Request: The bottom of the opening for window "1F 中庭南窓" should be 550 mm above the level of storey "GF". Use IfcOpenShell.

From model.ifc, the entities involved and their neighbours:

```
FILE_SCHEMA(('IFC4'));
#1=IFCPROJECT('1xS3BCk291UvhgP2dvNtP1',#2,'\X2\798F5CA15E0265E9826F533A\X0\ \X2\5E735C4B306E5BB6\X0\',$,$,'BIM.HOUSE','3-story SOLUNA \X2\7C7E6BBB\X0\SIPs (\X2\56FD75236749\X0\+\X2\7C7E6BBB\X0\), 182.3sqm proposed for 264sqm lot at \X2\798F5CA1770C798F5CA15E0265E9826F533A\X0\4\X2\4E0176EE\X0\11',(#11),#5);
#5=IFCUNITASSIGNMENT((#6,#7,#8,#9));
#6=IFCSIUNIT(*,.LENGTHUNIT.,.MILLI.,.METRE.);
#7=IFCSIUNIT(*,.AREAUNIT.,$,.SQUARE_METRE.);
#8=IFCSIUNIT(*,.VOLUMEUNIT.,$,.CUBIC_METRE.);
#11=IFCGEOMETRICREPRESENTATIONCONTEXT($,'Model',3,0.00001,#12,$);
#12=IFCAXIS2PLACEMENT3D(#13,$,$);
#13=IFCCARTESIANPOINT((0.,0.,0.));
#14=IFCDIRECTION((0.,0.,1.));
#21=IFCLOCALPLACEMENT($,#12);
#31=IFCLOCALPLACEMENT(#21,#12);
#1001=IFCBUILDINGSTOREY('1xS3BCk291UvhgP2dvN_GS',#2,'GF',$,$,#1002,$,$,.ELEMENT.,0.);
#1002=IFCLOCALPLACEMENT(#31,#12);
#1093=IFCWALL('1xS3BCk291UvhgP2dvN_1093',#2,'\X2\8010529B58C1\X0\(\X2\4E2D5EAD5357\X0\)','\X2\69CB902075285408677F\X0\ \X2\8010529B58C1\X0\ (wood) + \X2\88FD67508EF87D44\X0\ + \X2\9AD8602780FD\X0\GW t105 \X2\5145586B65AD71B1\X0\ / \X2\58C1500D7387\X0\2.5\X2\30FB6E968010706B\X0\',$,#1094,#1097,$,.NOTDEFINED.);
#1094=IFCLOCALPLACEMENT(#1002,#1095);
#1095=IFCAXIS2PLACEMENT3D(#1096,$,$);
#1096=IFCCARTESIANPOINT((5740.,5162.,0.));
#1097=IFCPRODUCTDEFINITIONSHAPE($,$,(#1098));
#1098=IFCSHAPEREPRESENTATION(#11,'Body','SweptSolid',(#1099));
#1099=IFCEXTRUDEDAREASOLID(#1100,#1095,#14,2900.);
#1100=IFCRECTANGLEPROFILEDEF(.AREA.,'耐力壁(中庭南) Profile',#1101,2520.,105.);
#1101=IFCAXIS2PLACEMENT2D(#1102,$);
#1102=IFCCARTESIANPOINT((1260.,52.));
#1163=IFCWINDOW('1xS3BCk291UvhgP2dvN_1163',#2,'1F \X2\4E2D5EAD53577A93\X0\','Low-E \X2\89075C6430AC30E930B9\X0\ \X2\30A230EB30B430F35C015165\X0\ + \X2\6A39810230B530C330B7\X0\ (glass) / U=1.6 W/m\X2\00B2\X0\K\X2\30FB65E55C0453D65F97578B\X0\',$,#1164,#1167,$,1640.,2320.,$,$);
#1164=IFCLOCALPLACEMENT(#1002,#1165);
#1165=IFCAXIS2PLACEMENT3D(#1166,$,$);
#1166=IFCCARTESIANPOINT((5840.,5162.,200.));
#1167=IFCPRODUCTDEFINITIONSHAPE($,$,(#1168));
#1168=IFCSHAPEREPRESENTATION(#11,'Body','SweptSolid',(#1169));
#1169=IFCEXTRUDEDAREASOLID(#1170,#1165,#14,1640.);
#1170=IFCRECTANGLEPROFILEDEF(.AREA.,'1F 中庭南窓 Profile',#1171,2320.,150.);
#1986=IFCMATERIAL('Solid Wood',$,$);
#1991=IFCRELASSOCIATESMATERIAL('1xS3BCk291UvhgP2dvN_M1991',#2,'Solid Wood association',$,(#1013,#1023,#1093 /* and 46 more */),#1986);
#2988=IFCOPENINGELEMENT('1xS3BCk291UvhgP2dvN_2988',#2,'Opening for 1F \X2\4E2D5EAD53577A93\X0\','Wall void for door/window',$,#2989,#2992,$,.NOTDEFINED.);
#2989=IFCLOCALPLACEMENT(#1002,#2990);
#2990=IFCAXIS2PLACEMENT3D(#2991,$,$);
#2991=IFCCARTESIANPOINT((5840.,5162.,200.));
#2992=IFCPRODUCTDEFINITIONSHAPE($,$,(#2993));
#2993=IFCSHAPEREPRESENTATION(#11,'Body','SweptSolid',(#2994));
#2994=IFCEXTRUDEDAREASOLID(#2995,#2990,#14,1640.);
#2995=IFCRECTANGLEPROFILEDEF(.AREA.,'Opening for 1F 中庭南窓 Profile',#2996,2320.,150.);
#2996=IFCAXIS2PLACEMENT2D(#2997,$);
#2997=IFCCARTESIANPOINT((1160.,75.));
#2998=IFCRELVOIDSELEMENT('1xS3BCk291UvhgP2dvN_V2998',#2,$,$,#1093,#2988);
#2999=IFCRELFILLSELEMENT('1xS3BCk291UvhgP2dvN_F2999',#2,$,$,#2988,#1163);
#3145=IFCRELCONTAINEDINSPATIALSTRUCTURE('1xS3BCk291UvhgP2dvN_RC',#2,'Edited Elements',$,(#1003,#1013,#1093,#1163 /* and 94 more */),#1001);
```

```python
import numpy as np
import ifcopenshell
import ifcopenshell.api.geometry
import ifcopenshell.geom
import ifcopenshell.util.element
import ifcopenshell.util.placement
import ifcopenshell.util.shape
import ifcopenshell.util.unit

model = ifcopenshell.open("model.ifc")
unit_scale = ifcopenshell.util.unit.calculate_unit_scale(model)

window = model.by_guid("1xS3BCk291UvhgP2dvN_1163")
opening = window.FillsVoids[0].RelatingOpeningElement
storey = ifcopenshell.util.element.get_container(window, ifc_class="IfcBuildingStorey")
level = ifcopenshell.util.placement.get_local_placement(storey.ObjectPlacement)[2, 3]

# The opening's origin need not be at the sill, so measure its lowest point.
shape = ifcopenshell.geom.create_shape(ifcopenshell.geom.settings(), opening)
bottom = ifcopenshell.util.shape.get_shape_bottom_elevation(shape, shape.geometry) / unit_scale
dz = level + 550.0 - bottom

shift = np.array([0.0, 0.0, dz])
# The window is not placed relative to its opening, so move both.
for product in (opening, window):
    matrix = ifcopenshell.util.placement.get_local_placement(product.ObjectPlacement)
    matrix[:3, 3] += shift
    ifcopenshell.api.geometry.edit_object_placement(model, product=product, matrix=matrix, is_si=False)

print(f"moved by {dz * unit_scale:+.3f} m")

model.write("model-out.ifc")
```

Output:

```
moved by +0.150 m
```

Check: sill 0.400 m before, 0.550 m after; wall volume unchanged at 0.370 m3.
